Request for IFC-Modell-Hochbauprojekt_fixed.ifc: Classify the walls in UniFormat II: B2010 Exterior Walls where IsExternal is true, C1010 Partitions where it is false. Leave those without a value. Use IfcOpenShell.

First a look at what the model holds.

```python
import ifcopenshell
import ifcopenshell.util.element

model = ifcopenshell.open("IFC-Modell-Hochbauprojekt_fixed.ifc")
print(model.schema)
print("classifications:", [c.Name for c in model.by_type("IfcClassification")])
values = [ifcopenshell.util.element.get_pset(e, "Pset_WallCommon", "IsExternal") for e in model.by_type("IfcWall")]
for value in (True, False, None):
    print("IsExternal", value, values.count(value))
```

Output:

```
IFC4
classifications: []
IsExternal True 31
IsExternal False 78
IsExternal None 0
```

```python
import ifcopenshell
import ifcopenshell.api.classification
import ifcopenshell.util.element

model = ifcopenshell.open("IFC-Modell-Hochbauprojekt_fixed.ifc")

system = ifcopenshell.api.classification.add_classification(model, classification="UniFormat II")

walls = model.by_type("IfcWall")
external = {e: ifcopenshell.util.element.get_pset(e, "Pset_WallCommon", "IsExternal") for e in walls}
for flag, code, name in ((True, "B2010", "Exterior Walls"), (False, "C1010", "Partitions")):
    products = [e for e in walls if external[e] is flag]
    ifcopenshell.api.classification.add_reference(
        model, products=products, classification=system, identification=code, name=name
    )
    print(code, len(products))

model.write("IFC-Modell-Hochbauprojekt_fixed_edited.ifc")
```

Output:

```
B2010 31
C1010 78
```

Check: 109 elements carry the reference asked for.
